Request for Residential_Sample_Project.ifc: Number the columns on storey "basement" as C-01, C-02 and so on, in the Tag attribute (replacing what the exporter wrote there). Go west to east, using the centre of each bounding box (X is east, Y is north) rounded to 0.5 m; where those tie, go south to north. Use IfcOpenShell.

First a look at what the model holds.

```python
import ifcopenshell
import ifcopenshell.util.element
import ifcopenshell.util.placement

model = ifcopenshell.open("Residential_Sample_Project.ifc")
print(model.schema)
storey = next(s for s in model.by_type("IfcBuildingStorey") if s.Name == "basement")
columns = [e for e in ifcopenshell.util.element.get_decomposition(storey) if e.is_a("IfcColumn")]
for e in sorted(columns, key=lambda e: e.id()):
    origin = ifcopenshell.util.placement.get_local_placement(e.ObjectPlacement)[:3, 3]
    print(e.id(), e.Tag, e.Name, origin.round(2) + 0.0, sep=" | ")
```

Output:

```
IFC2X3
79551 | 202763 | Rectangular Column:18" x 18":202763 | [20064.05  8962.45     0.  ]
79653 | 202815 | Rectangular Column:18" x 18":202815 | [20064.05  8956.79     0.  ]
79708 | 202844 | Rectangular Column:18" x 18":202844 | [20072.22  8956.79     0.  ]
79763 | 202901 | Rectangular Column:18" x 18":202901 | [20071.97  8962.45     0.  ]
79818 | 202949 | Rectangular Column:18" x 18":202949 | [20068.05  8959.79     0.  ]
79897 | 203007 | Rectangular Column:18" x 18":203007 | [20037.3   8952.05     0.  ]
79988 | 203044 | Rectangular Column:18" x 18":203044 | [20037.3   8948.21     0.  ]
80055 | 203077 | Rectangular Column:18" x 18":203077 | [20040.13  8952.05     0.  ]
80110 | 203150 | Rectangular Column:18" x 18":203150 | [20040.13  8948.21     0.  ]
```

```python
import ifcopenshell
import ifcopenshell.geom
import ifcopenshell.util.element
import ifcopenshell.util.shape

model = ifcopenshell.open("Residential_Sample_Project.ifc")
settings = ifcopenshell.geom.settings()
settings.set("use-world-coords", True)


def centre(element):
    shape = ifcopenshell.geom.create_shape(settings, element)
    return ifcopenshell.util.shape.get_bbox_centroid(shape.geometry)


storey = next(s for s in model.by_type("IfcBuildingStorey") if s.Name == "basement")
columns = [e for e in ifcopenshell.util.element.get_decomposition(storey) if e.is_a("IfcColumn")]

# Insertion points can sit at a corner or the storey origin, so sort by the geometry (in metres).
centres = {e: centre(e) for e in columns}
columns.sort(key=lambda e: (round(centres[e][0] / 0.5), centres[e][1]))

for i, e in enumerate(columns, start=1):
    number = f"C-{i:02d}"
    e.Tag = number
    print(e.id(), number)

model.write("Residential_Sample_Project_v2.ifc")
```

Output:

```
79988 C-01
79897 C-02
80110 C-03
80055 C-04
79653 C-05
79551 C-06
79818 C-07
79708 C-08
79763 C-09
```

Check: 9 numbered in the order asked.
